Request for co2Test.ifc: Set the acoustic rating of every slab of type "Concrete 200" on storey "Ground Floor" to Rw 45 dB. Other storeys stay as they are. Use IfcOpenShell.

First a look at what the model holds.

```python
import ifcopenshell
import ifcopenshell.util.element

model = ifcopenshell.open("co2Test.ifc")
print(model.schema)
storey = next(s for s in model.by_type("IfcBuildingStorey") if s.Name == "Ground Floor")
slabs = [e for e in ifcopenshell.util.element.get_decomposition(storey) if e.is_a("IfcSlab")]
seen = {}
for e in slabs:
    element_type = ifcopenshell.util.element.get_type(e)
    key = (element_type.Name if element_type != e and element_type else None, ifcopenshell.util.element.get_pset(e, "Pset_SlabCommon", "AcousticRating"))
    seen[key] = seen.get(key, 0) + 1
for (name, value), count in sorted(seen.items(), key=str):
    print(count, "x", name, "|", value)
```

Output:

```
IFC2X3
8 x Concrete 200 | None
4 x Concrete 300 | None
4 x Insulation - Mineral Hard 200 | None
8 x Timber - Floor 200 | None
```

```python
import ifcopenshell
import ifcopenshell.api.pset
import ifcopenshell.util.element

model = ifcopenshell.open("co2Test.ifc")

storey = next(s for s in model.by_type("IfcBuildingStorey") if s.Name == "Ground Floor")
slabs = [e for e in ifcopenshell.util.element.get_decomposition(storey) if e.is_a("IfcSlab")]

count = 0
for e in slabs:
    element_type = ifcopenshell.util.element.get_type(e)
    if element_type in (None, e) or element_type.Name != "Concrete 200":
        continue
    # add_pset returns the element's existing set when there is one.
    pset = ifcopenshell.api.pset.add_pset(model, product=e, name="Pset_SlabCommon")
    ifcopenshell.api.pset.edit_pset(model, pset=pset, properties={"AcousticRating": "Rw 45 dB"})
    count += 1

print(count, "slabs updated")

model.write("co2Test_edited.ifc")
```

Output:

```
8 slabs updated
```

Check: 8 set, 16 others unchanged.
